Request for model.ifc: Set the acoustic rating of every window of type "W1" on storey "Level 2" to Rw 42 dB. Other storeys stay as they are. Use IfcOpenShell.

First a look at what the model holds.

```python
import ifcopenshell
import ifcopenshell.util.element

model = ifcopenshell.open("model.ifc")
print(model.schema)
storey = next(s for s in model.by_type("IfcBuildingStorey") if s.Name == "Level 2")
windows = [e for e in ifcopenshell.util.element.get_decomposition(storey) if e.is_a("IfcWindow")]
seen = {}
for e in windows:
    element_type = ifcopenshell.util.element.get_type(e)
    key = (element_type.Name if element_type != e and element_type else None, ifcopenshell.util.element.get_pset(e, "Pset_WindowCommon", "AcousticRating"))
    seen[key] = seen.get(key, 0) + 1
for (name, value), count in sorted(seen.items(), key=str):
    print(count, "x", name, "|", value)
```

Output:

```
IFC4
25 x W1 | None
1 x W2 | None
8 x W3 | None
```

```python
import ifcopenshell
import ifcopenshell.api.pset
import ifcopenshell.util.element

model = ifcopenshell.open("model.ifc")

storey = next(s for s in model.by_type("IfcBuildingStorey") if s.Name == "Level 2")
windows = [e for e in ifcopenshell.util.element.get_decomposition(storey) if e.is_a("IfcWindow")]

count = 0
for e in windows:
    element_type = ifcopenshell.util.element.get_type(e)
    if element_type in (None, e) or element_type.Name != "W1":
        continue
    # add_pset returns the element's existing set when there is one.
    pset = ifcopenshell.api.pset.add_pset(model, product=e, name="Pset_WindowCommon")
    ifcopenshell.api.pset.edit_pset(model, pset=pset, properties={"AcousticRating": "Rw 42 dB"})
    count += 1

print(count, "windows updated")

model.write("model-out.ifc")
```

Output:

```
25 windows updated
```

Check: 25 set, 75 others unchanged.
